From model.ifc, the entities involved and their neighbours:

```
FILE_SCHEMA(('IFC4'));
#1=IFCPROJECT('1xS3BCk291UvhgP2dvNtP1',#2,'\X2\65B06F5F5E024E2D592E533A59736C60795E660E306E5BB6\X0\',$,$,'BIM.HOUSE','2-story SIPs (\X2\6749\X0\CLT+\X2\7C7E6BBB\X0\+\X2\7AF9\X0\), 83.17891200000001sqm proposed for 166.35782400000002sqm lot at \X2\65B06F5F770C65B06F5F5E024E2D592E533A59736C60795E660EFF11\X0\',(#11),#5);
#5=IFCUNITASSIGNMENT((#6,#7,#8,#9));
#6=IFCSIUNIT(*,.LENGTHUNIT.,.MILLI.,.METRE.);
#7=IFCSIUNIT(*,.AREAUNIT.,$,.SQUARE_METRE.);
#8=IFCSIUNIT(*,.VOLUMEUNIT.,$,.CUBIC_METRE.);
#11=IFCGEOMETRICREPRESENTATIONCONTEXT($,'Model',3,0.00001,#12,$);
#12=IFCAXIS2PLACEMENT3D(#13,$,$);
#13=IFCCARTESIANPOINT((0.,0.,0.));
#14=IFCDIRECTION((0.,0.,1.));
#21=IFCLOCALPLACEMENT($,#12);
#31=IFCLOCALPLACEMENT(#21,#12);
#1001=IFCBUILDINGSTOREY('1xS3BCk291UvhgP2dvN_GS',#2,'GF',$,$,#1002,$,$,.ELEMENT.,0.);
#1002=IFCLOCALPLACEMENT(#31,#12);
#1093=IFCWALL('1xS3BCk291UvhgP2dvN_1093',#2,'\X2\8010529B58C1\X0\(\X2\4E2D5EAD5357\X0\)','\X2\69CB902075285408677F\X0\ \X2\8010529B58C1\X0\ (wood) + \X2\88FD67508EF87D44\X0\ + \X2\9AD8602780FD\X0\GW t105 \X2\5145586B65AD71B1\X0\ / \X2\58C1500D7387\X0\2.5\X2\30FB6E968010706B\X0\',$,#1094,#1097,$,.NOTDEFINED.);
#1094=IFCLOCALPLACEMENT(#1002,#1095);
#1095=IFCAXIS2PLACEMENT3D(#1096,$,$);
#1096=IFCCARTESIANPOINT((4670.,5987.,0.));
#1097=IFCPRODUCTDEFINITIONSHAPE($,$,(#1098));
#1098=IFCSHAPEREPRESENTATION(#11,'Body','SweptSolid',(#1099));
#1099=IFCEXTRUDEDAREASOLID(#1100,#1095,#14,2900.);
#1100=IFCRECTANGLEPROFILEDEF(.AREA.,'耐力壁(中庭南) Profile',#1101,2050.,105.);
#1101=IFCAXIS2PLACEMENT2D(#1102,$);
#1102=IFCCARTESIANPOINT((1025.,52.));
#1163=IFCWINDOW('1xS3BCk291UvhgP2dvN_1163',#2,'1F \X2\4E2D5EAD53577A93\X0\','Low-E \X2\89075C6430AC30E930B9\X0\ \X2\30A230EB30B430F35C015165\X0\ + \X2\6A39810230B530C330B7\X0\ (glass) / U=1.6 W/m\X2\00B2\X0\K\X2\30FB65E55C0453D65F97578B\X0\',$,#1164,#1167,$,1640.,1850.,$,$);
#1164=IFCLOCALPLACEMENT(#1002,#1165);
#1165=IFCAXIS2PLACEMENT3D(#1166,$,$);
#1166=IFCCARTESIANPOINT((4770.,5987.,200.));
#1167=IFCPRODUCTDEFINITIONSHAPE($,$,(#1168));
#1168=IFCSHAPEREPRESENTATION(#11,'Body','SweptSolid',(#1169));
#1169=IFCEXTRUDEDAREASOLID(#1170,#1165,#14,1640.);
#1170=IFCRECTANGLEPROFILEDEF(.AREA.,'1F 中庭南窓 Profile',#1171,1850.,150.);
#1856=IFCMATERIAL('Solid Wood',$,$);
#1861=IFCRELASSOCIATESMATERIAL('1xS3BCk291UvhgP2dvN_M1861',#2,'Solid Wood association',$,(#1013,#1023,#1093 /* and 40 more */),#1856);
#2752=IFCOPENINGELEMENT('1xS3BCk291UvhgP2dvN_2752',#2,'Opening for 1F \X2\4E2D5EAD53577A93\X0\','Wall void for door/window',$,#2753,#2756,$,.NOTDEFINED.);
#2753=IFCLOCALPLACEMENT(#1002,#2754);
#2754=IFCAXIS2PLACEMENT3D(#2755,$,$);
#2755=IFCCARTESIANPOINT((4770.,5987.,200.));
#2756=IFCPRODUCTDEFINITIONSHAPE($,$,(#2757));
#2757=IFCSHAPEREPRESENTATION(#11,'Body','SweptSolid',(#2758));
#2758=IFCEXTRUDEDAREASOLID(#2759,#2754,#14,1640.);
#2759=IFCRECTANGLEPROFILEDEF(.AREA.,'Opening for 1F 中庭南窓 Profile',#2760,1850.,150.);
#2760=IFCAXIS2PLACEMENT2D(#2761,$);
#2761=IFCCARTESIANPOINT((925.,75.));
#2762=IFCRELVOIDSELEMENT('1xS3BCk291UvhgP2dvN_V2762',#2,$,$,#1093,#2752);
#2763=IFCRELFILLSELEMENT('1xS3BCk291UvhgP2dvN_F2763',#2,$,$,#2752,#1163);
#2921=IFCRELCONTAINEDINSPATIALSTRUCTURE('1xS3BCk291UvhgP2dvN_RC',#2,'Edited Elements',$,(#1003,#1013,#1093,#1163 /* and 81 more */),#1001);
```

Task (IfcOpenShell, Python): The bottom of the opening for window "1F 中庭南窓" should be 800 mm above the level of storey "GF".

```python
import numpy as np
import ifcopenshell
import ifcopenshell.api.geometry
import ifcopenshell.geom
import ifcopenshell.util.element
import ifcopenshell.util.placement
import ifcopenshell.util.shape
import ifcopenshell.util.unit

model = ifcopenshell.open("model.ifc")
unit_scale = ifcopenshell.util.unit.calculate_unit_scale(model)

window = model.by_guid("1xS3BCk291UvhgP2dvN_1163")
opening = window.FillsVoids[0].RelatingOpeningElement
storey = ifcopenshell.util.element.get_container(window, ifc_class="IfcBuildingStorey")
level = ifcopenshell.util.placement.get_local_placement(storey.ObjectPlacement)[2, 3]

# The opening's origin need not be at the sill, so measure its lowest point.
shape = ifcopenshell.geom.create_shape(ifcopenshell.geom.settings(), opening)
bottom = ifcopenshell.util.shape.get_shape_bottom_elevation(shape, shape.geometry) / unit_scale
dz = level + 0.8 / unit_scale - bottom

shift = np.array([0.0, 0.0, dz])
# The window is not placed relative to its opening, so move both.
for product in (opening, window):
    matrix = ifcopenshell.util.placement.get_local_placement(product.ObjectPlacement)
    matrix[:3, 3] += shift
    ifcopenshell.api.geometry.edit_object_placement(model, product=product, matrix=matrix, is_si=False)

print(f"moved by {dz * unit_scale:+.3f} m")

model.write("model_rev.ifc")
```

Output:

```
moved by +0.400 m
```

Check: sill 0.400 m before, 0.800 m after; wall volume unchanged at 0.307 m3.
